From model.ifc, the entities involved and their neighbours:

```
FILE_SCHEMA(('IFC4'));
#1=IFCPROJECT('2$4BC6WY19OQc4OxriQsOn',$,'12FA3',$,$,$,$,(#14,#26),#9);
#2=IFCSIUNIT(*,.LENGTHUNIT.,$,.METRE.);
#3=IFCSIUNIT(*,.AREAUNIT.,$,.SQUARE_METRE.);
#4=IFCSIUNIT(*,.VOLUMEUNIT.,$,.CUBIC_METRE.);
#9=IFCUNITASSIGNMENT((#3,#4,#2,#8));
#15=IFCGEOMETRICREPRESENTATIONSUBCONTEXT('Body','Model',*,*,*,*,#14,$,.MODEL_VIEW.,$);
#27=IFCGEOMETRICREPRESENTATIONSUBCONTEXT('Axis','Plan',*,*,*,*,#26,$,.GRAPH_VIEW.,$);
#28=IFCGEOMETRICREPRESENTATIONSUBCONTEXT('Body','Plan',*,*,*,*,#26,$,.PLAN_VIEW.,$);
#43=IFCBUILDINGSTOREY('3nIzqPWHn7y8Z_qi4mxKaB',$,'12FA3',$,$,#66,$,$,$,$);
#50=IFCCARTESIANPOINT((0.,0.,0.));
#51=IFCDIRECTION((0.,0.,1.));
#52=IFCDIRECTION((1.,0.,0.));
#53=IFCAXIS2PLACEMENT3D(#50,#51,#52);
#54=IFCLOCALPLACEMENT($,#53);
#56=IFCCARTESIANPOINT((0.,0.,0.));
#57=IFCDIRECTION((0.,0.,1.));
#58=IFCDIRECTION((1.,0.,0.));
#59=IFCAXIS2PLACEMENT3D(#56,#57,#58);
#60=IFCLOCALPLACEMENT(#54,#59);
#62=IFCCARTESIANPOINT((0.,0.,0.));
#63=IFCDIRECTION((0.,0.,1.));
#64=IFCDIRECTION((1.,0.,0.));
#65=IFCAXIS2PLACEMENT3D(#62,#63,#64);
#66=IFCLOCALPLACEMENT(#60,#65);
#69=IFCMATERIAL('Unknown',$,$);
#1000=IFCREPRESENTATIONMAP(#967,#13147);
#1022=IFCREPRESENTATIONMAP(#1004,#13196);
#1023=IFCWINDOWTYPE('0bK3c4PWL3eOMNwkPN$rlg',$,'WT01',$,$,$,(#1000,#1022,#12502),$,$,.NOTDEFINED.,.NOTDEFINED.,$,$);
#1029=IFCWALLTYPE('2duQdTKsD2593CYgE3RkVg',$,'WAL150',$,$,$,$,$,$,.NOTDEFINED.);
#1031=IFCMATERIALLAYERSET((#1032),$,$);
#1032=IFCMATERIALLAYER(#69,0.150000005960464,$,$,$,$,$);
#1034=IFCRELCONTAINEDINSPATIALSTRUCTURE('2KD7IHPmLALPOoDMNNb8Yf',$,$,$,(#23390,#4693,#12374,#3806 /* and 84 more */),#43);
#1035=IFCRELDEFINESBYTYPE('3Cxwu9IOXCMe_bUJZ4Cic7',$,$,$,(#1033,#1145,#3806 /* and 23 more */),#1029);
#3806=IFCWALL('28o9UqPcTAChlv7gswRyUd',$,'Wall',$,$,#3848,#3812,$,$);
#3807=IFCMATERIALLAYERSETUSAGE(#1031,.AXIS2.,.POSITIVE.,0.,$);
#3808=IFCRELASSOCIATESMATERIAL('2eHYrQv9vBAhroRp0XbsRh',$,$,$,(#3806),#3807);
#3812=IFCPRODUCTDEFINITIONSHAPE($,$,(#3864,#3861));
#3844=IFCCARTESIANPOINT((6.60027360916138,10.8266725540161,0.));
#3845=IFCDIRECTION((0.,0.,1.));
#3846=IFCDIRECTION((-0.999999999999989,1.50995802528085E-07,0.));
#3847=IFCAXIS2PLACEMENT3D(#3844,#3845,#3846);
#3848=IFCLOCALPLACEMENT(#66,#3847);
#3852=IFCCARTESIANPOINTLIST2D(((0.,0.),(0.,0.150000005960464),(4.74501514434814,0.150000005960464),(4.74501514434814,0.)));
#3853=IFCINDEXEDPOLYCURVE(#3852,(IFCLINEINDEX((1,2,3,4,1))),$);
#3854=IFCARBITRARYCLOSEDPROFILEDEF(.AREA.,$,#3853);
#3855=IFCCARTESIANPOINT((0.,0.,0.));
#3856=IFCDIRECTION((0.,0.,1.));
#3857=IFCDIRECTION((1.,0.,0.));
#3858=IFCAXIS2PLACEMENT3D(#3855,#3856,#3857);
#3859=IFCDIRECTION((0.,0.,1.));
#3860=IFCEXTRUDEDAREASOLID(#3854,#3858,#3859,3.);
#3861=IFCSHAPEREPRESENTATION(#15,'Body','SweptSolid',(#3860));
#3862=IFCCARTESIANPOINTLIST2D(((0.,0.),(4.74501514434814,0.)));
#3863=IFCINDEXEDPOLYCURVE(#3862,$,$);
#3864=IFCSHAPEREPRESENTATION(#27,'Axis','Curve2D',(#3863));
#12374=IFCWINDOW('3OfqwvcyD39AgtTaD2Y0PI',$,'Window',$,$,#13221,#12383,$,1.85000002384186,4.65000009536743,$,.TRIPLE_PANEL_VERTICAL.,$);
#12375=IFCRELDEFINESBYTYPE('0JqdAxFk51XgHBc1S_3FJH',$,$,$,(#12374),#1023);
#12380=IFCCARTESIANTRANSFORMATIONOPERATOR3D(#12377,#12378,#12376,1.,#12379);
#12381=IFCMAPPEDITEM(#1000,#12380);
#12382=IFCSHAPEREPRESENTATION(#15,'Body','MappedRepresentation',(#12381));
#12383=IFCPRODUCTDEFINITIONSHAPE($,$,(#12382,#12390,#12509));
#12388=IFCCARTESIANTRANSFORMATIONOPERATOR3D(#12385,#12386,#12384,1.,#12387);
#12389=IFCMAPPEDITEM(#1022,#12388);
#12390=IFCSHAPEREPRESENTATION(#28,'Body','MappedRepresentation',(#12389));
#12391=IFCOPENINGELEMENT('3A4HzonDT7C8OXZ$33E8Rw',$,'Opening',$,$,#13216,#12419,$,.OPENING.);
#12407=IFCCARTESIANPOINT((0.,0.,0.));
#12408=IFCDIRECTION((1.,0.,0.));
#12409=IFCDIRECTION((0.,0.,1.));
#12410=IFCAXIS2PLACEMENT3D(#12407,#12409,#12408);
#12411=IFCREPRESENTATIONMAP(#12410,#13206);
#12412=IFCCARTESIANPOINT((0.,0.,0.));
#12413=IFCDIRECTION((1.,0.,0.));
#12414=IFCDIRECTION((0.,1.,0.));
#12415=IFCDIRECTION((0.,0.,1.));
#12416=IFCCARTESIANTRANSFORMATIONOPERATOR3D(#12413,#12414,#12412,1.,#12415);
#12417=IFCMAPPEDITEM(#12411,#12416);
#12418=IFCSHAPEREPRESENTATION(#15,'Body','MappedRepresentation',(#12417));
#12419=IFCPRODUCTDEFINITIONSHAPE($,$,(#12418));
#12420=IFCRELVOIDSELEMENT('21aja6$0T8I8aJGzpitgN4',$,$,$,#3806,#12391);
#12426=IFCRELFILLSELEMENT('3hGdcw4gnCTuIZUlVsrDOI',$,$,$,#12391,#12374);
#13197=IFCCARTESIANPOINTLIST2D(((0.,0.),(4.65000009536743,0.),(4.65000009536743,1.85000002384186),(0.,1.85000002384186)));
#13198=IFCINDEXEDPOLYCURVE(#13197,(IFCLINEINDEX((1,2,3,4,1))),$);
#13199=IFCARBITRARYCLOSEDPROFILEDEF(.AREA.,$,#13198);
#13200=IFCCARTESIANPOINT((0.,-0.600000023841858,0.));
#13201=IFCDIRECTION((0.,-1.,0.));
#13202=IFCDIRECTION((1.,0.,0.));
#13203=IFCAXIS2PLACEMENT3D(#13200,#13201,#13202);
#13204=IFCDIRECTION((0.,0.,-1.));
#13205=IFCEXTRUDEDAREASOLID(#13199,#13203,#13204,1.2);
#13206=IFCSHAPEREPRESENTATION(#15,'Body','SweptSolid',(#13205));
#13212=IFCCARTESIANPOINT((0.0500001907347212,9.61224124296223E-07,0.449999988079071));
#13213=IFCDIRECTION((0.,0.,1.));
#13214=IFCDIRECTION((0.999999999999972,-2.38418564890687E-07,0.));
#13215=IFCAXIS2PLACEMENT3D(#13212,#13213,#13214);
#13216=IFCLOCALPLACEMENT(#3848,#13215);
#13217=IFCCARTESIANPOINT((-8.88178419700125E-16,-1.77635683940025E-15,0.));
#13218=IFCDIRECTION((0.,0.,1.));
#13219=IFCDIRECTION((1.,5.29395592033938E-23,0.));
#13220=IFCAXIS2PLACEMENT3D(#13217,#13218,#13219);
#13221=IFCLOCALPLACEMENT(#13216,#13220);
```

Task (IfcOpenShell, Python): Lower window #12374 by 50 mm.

```python
import numpy as np
import ifcopenshell
import ifcopenshell.api.geometry
import ifcopenshell.util.placement
import ifcopenshell.util.unit

model = ifcopenshell.open("model.ifc")
unit_scale = ifcopenshell.util.unit.calculate_unit_scale(model)

window = model.by_guid("3OfqwvcyD39AgtTaD2Y0PI")
opening = window.FillsVoids[0].RelatingOpeningElement
dz = -0.05 / unit_scale

shift = np.array([0.0, 0.0, dz])
# The window is placed relative to its opening, so it follows when the opening moves.
matrix = ifcopenshell.util.placement.get_local_placement(opening.ObjectPlacement)
matrix[:3, 3] += shift
ifcopenshell.api.geometry.edit_object_placement(
    model, product=opening, matrix=matrix, is_si=False, should_transform_children=True
)

print(f"moved by {dz * unit_scale:+.3f} m")

model.write("model_rev.ifc")
```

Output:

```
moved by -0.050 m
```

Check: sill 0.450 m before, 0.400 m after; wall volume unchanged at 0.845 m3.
